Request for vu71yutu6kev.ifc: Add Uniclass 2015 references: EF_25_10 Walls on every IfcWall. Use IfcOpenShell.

First a look at what the model holds.

```python
import ifcopenshell

model = ifcopenshell.open("vu71yutu6kev.ifc")
print(model.schema)
print("classifications:", [c.Name for c in model.by_type("IfcClassification")])
for ifc_class in ("IfcDoor", "IfcRoof", "IfcStair", "IfcWall", "IfcWindow"):
    print(ifc_class, len(model.by_type(ifc_class)))
```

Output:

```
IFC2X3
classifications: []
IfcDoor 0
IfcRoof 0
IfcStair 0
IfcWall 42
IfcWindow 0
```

```python
import ifcopenshell
import ifcopenshell.api.classification

model = ifcopenshell.open("vu71yutu6kev.ifc")

# IFC2X3 requires Source and Edition and has no link from the project to the system.
system = model.create_entity("IfcClassification", Source="NBS", Edition="2015", Name="Uniclass 2015")

codes = {
    "IfcWall": ("EF_25_10", "Walls"),
}
for ifc_class, (code, name) in codes.items():
    products = model.by_type(ifc_class)
    ifcopenshell.api.classification.add_reference(
        model, products=products, classification=system, identification=code, name=name
    )
    print(code, len(products))

model.write("vu71yutu6kev_updated.ifc")
```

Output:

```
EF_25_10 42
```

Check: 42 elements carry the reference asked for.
